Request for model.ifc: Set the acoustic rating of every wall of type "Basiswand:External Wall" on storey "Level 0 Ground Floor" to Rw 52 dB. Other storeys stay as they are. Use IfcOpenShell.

First a look at what the model holds.

```python
import ifcopenshell
import ifcopenshell.util.element

model = ifcopenshell.open("model.ifc")
print(model.schema)
storey = next(s for s in model.by_type("IfcBuildingStorey") if s.Name == "Level 0 Ground Floor")
walls = [e for e in ifcopenshell.util.element.get_decomposition(storey) if e.is_a("IfcWall")]
seen = {}
for e in walls:
    element_type = ifcopenshell.util.element.get_type(e)
    key = (element_type.Name if element_type != e and element_type else None, ifcopenshell.util.element.get_pset(e, "Pset_WallCommon", "AcousticRating"))
    seen[key] = seen.get(key, 0) + 1
for (name, value), count in sorted(seen.items(), key=str):
    print(count, "x", name, "|", value)
```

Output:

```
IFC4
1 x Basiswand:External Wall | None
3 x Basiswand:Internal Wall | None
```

```python
import ifcopenshell
import ifcopenshell.api.pset
import ifcopenshell.util.element

model = ifcopenshell.open("model.ifc")

storey = next(s for s in model.by_type("IfcBuildingStorey") if s.Name == "Level 0 Ground Floor")
walls = [e for e in ifcopenshell.util.element.get_decomposition(storey) if e.is_a("IfcWall")]

count = 0
for e in walls:
    element_type = ifcopenshell.util.element.get_type(e)
    if element_type in (None, e) or element_type.Name != "Basiswand:External Wall":
        continue
    # add_pset returns the element's existing set when there is one.
    pset = ifcopenshell.api.pset.add_pset(model, product=e, name="Pset_WallCommon")
    ifcopenshell.api.pset.edit_pset(model, pset=pset, properties={"AcousticRating": "Rw 52 dB"})
    count += 1

print(count, "walls updated")

model.write("model-out.ifc")
```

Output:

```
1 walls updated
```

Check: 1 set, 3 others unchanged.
